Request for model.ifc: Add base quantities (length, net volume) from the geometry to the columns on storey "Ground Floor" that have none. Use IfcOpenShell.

First a look at what the model holds.

```python
import ifcopenshell
import ifcopenshell.util.element
import ifcopenshell.util.unit

model = ifcopenshell.open("model.ifc")
print(model.schema)
for unit_type in ("LENGTHUNIT", "AREAUNIT", "VOLUMEUNIT"):
    print(unit_type, ifcopenshell.util.unit.calculate_unit_scale(model, unit_type))
storey = next(s for s in model.by_type("IfcBuildingStorey") if s.Name == "Ground Floor")
columns = [e for e in ifcopenshell.util.element.get_decomposition(storey) if e.is_a("IfcColumn")]
for e in sorted(columns, key=lambda e: e.id()):
    print(e.id(), e.is_a(), e.Name, list(ifcopenshell.util.element.get_psets(e, qtos_only=True)), sep=" | ")
```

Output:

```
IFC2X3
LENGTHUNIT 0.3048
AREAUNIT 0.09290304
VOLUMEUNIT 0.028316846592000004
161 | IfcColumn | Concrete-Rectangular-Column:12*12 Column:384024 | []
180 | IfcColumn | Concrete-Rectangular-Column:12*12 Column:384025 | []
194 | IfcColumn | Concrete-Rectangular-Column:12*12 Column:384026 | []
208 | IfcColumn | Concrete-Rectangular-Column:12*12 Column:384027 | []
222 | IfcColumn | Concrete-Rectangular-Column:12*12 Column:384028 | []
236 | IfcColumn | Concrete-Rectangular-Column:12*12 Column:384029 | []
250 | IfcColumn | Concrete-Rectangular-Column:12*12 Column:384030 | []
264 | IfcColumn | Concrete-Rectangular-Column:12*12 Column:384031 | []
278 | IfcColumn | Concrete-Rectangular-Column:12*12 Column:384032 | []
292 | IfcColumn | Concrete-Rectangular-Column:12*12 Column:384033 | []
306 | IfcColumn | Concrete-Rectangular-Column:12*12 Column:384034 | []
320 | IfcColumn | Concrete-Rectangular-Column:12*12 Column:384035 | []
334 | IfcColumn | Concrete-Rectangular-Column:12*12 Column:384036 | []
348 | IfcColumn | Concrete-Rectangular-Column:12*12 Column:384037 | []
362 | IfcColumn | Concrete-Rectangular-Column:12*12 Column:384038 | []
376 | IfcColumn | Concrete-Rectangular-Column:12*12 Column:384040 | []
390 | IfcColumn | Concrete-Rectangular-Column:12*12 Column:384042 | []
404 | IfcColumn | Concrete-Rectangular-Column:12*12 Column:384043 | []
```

```python
import ifcopenshell
import ifcopenshell.api.pset
import ifcopenshell.geom
import ifcopenshell.util.element
import ifcopenshell.util.shape
import ifcopenshell.util.unit

model = ifcopenshell.open("model.ifc")
unit_scale = ifcopenshell.util.unit.calculate_unit_scale(model)
volume_scale = ifcopenshell.util.unit.calculate_unit_scale(model, "VOLUMEUNIT")
settings = ifcopenshell.geom.settings()

storey = next(s for s in model.by_type("IfcBuildingStorey") if s.Name == "Ground Floor")
columns = [e for e in ifcopenshell.util.element.get_decomposition(storey) if e.is_a("IfcColumn")]

for e in sorted(columns, key=lambda e: e.id()):
    if ifcopenshell.util.element.get_psets(e, qtos_only=True, should_inherit=False):
        continue
    # Geometry comes back in metres, in the element's own axes.
    shape = ifcopenshell.geom.create_shape(settings, e)
    values = {
        "Length": ifcopenshell.util.shape.get_z(shape.geometry) / unit_scale,
        "NetVolume": ifcopenshell.util.shape.get_volume(shape.geometry) / volume_scale,
    }
    qto = ifcopenshell.api.pset.add_qto(model, product=e, name="BaseQuantities")
    ifcopenshell.api.pset.edit_qto(model, qto=qto, properties=values)
    print(e.id(), {k: round(v, 3) for k, v in values.items()})

model.write("model-out.ifc")
```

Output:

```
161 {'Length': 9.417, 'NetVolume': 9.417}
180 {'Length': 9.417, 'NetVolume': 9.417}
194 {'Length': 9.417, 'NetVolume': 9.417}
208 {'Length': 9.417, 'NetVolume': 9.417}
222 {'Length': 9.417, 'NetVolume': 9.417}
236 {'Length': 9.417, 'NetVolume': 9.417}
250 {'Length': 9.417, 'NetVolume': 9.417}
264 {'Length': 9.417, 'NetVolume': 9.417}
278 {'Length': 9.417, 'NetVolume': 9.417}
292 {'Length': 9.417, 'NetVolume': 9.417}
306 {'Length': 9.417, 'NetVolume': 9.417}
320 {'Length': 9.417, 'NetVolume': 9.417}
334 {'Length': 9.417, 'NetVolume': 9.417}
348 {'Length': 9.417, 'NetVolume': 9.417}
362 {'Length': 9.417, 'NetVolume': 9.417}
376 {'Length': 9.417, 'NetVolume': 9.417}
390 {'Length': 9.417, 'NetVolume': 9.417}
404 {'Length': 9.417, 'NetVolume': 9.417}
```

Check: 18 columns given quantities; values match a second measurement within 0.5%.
